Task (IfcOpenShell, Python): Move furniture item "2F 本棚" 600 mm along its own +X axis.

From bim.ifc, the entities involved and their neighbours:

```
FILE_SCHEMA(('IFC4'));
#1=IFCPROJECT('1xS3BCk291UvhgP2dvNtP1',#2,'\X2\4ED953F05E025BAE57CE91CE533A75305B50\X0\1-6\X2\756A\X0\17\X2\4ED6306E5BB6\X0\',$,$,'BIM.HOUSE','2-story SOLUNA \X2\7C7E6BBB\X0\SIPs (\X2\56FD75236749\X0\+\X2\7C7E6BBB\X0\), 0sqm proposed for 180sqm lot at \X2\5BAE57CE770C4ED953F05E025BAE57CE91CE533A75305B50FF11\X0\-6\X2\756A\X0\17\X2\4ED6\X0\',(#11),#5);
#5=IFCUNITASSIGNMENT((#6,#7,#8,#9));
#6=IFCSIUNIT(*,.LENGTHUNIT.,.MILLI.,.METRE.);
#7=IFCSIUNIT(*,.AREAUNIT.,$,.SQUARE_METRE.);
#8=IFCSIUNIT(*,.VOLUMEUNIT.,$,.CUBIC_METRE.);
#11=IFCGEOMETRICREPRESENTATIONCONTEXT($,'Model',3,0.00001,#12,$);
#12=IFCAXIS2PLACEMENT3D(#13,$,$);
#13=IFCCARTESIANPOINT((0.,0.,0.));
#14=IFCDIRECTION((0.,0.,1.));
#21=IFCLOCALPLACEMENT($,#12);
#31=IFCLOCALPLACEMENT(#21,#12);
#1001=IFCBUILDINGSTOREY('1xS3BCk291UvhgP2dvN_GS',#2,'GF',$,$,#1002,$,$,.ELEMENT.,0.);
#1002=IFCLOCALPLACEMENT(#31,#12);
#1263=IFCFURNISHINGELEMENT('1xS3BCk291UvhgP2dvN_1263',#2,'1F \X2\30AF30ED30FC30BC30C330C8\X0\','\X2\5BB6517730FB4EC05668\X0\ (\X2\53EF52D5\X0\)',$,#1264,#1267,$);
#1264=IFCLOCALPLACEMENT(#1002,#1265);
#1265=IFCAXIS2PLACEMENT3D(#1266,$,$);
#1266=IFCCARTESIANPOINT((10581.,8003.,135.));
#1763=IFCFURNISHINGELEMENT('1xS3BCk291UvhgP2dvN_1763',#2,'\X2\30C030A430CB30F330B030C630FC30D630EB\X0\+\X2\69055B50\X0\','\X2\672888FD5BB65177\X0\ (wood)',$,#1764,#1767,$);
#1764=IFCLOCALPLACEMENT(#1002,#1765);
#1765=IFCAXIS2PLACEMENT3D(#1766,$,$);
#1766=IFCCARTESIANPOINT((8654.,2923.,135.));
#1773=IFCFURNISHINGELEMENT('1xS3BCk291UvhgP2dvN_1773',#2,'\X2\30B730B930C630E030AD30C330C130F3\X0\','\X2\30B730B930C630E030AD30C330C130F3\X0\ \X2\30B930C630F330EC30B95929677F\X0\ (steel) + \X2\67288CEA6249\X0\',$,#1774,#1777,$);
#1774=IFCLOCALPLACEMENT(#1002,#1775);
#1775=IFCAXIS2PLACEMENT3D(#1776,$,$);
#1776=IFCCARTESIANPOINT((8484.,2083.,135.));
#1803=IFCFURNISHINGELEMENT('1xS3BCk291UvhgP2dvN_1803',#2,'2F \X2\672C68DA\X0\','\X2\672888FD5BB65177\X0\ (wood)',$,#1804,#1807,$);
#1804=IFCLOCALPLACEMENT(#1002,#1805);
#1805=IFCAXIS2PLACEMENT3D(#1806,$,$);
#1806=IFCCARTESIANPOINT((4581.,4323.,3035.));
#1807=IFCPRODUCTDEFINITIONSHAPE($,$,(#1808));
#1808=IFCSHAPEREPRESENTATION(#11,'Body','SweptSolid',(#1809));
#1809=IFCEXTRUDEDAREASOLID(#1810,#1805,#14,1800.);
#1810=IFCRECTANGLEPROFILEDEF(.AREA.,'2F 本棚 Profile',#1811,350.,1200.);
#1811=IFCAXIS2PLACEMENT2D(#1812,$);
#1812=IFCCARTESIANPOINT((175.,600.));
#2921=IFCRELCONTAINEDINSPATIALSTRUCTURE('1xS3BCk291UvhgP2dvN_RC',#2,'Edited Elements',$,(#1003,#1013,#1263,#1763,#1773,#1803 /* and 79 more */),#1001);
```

```python
import ifcopenshell
import ifcopenshell.api.geometry
import ifcopenshell.util.placement

model = ifcopenshell.open("bim.ifc")

item = model.by_guid("1xS3BCk291UvhgP2dvN_1803")
matrix = ifcopenshell.util.placement.get_local_placement(item.ObjectPlacement)
matrix[:3, 3] += matrix[:3, 0] * 600.0
ifcopenshell.api.geometry.edit_object_placement(model, product=item, matrix=matrix, is_si=False)

print(ifcopenshell.util.placement.get_local_placement(item.ObjectPlacement).round(3) + 0.0)

model.write("bim_rev.ifc")
```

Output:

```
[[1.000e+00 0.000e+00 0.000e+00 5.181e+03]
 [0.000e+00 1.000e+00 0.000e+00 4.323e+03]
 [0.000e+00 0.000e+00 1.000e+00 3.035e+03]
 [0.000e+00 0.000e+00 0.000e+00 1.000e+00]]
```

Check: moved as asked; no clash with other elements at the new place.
